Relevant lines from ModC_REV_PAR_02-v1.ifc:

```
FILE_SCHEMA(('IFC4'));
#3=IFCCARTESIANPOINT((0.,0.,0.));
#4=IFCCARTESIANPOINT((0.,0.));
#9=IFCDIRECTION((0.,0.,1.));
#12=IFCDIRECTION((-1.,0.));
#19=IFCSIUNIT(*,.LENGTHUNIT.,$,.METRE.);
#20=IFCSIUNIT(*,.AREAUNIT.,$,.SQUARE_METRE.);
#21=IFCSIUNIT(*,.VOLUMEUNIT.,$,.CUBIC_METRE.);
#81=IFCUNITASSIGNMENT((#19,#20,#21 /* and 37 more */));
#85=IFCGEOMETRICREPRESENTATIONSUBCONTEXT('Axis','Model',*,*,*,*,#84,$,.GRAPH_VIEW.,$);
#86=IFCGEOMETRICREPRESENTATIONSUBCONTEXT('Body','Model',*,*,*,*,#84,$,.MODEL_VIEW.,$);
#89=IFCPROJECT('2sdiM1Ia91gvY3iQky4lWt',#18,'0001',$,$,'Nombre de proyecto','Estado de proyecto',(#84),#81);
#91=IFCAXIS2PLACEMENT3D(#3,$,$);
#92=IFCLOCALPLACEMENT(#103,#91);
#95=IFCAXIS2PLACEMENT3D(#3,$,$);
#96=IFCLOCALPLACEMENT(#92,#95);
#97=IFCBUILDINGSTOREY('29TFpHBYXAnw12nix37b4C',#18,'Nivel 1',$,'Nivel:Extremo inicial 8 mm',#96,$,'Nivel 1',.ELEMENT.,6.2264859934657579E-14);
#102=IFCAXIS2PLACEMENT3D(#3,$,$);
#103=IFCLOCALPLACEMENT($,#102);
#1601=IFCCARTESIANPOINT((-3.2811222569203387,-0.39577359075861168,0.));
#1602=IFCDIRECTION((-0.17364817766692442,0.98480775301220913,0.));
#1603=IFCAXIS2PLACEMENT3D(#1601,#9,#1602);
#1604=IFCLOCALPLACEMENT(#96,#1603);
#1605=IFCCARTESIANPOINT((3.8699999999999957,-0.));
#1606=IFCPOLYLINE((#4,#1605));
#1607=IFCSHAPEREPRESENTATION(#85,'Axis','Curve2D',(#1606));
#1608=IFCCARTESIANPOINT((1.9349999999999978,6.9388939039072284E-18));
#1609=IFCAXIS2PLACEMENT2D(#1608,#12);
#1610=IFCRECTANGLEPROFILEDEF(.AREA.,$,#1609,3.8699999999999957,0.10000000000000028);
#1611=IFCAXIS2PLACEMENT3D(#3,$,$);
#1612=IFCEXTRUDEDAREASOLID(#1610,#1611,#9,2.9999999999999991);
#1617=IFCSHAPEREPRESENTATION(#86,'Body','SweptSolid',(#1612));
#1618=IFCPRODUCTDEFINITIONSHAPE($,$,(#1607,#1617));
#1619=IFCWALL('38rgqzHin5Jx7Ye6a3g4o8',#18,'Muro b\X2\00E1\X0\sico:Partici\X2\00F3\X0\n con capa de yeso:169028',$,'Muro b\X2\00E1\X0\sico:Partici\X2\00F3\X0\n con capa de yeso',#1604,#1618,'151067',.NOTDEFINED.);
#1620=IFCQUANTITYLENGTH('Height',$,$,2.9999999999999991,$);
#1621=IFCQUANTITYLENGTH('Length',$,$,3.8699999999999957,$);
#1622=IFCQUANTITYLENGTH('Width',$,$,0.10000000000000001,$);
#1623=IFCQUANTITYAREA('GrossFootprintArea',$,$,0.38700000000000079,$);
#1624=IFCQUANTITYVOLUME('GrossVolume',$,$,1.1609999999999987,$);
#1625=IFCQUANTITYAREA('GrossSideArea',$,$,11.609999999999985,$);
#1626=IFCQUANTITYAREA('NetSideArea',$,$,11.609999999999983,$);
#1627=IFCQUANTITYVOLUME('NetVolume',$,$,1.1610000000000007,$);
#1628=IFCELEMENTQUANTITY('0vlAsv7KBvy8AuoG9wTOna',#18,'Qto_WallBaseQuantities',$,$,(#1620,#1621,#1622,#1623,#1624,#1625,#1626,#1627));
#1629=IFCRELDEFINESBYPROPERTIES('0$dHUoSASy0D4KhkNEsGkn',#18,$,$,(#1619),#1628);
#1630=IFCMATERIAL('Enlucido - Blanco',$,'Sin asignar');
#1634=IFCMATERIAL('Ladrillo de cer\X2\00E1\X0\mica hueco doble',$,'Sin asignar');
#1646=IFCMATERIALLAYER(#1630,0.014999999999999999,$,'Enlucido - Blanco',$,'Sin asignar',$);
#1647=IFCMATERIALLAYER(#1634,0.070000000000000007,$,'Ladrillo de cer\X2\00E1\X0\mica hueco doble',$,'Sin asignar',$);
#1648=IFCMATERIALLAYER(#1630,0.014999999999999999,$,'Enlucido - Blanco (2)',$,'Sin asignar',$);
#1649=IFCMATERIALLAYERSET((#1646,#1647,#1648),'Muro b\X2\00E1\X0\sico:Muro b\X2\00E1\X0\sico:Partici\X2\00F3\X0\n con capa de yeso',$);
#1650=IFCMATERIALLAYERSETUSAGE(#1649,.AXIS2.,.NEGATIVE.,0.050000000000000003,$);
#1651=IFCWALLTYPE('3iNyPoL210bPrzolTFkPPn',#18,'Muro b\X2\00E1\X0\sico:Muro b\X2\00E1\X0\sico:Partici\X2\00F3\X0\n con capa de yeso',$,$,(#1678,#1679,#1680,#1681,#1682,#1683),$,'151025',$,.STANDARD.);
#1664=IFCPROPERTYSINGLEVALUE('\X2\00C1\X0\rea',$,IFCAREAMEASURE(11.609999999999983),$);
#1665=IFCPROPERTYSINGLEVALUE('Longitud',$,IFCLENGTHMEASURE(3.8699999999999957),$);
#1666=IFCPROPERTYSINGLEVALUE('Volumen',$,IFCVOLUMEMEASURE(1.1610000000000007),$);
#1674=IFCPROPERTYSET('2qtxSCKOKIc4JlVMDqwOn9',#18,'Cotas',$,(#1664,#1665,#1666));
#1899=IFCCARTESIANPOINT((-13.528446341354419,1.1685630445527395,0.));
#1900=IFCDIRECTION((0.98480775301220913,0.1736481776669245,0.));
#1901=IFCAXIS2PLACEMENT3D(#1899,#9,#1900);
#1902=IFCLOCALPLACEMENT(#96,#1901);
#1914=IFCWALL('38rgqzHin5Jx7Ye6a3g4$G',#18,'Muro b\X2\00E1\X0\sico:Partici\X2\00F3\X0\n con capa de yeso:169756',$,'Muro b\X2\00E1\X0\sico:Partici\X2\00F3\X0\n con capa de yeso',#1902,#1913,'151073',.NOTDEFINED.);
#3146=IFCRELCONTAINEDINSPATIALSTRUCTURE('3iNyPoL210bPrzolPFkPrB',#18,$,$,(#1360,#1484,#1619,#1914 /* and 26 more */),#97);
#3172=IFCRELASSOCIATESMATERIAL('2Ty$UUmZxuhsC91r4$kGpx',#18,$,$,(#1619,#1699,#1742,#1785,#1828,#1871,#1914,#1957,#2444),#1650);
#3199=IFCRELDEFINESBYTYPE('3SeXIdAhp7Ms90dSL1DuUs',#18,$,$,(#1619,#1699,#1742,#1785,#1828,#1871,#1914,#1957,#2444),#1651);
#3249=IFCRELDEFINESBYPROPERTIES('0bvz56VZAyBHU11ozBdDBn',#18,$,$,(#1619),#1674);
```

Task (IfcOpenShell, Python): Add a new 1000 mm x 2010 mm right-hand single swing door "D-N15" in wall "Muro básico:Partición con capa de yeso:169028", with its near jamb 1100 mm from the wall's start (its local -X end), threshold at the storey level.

```python
import numpy as np
import ifcopenshell
import ifcopenshell.api.feature
import ifcopenshell.api.geometry
import ifcopenshell.api.pset
import ifcopenshell.api.root
import ifcopenshell.api.spatial
import ifcopenshell.geom
import ifcopenshell.util.element
import ifcopenshell.util.placement
import ifcopenshell.util.representation
import ifcopenshell.util.shape
import ifcopenshell.util.unit

model = ifcopenshell.open("ModC_REV_PAR_02-v1.ifc")
unit_scale = ifcopenshell.util.unit.calculate_unit_scale(model)
area_scale = ifcopenshell.util.unit.calculate_unit_scale(model, "AREAUNIT")
volume_scale = ifcopenshell.util.unit.calculate_unit_scale(model, "VOLUMEUNIT")
settings = ifcopenshell.geom.settings()


def volume(element):
    """Net volume in cubic metres, openings subtracted."""
    shape = ifcopenshell.geom.create_shape(settings, element)
    return ifcopenshell.util.shape.get_volume(shape.geometry)


wall = model.by_guid("38rgqzHin5Jx7Ye6a3g4o8")
storey = ifcopenshell.util.element.get_container(wall, ifc_class="IfcBuildingStorey")
context = ifcopenshell.util.representation.get_context(model, "Model", "Body", "MODEL_VIEW")
before = volume(wall)

width, height, from_end, sill = 1, 2.01, 1.1, 0.0  # metres

# The wall runs along its own X axis, and the end named is its -X end.
wall_shape = ifcopenshell.geom.create_shape(settings, wall)
x, y, z = ifcopenshell.util.shape.get_vertices(wall_shape.geometry).T
start = x.min() + from_end
face, thickness = float(y.min()), float(y.max() - y.min())
wall_matrix = ifcopenshell.util.placement.get_local_placement(wall.ObjectPlacement)
level = ifcopenshell.util.placement.get_local_placement(storey.ObjectPlacement)[2, 3]


def in_wall(x, y):
    """Placement at x, y metres in the wall's axes, at sill height."""
    matrix = wall_matrix.copy()
    matrix[:, 3] = wall_matrix @ np.array([x / unit_scale, y / unit_scale, 0.0, 1.0])
    matrix[2, 3] = level + sill / unit_scale
    return matrix


# Opening: a box that overshoots both wall faces by 50 mm.
opening = ifcopenshell.api.root.create_entity(model, ifc_class="IfcOpeningElement", predefined_type="OPENING")
box = ifcopenshell.api.geometry.add_wall_representation(
    model, context=context, length=width, height=height, thickness=thickness + 0.1
)
ifcopenshell.api.geometry.assign_representation(model, product=opening, representation=box)
ifcopenshell.api.geometry.edit_object_placement(model, product=opening, matrix=in_wall(start, face - 0.05), is_si=False)
ifcopenshell.api.feature.add_feature(model, feature=opening, element=wall)

door = ifcopenshell.api.root.create_entity(model, ifc_class="IfcDoor", name="D-N15", predefined_type="DOOR")
door.OverallWidth, door.OverallHeight = width / unit_scale, height / unit_scale
door.OperationType = "SINGLE_SWING_RIGHT"
body = ifcopenshell.api.geometry.add_door_representation(
    model,
    context=context,
    overall_width=door.OverallWidth,
    overall_height=door.OverallHeight,
    operation_type="SINGLE_SWING_RIGHT",
    lining_properties={"LiningDepth": thickness / unit_scale, "ThresholdDepth": thickness / unit_scale},
)
ifcopenshell.api.geometry.assign_representation(model, product=door, representation=body)
ifcopenshell.api.spatial.assign_container(model, products=[door], relating_structure=storey)
ifcopenshell.api.feature.add_filling(model, opening=opening, element=door)

# The lining spans the wall, so the door starts at the wall face.
ifcopenshell.api.geometry.edit_object_placement(model, product=door, matrix=in_wall(start, face), is_si=False)

after = volume(wall)

# Update the wall's stored quantities.
qto = model.by_id(ifcopenshell.util.element.get_pset(wall, "Qto_WallBaseQuantities", should_inherit=False)["id"])
ifcopenshell.api.pset.edit_qto(model, qto=qto, properties={
    "NetSideArea": after / thickness / area_scale,
    "NetVolume": after / volume_scale,
})
pset = model.by_id(ifcopenshell.util.element.get_pset(wall, "Cotas", should_inherit=False)["id"])
ifcopenshell.api.pset.edit_pset(model, pset=pset, properties={
    "Área": model.create_entity("IfcAreaMeasure", after / thickness / area_scale),
    "Volumen": model.create_entity("IfcVolumeMeasure", after / volume_scale),
})

print(f"wall volume {before:.3f} -> {after:.3f} m3")

model.write("ModC_REV_PAR_02-v1_v2.ifc")
```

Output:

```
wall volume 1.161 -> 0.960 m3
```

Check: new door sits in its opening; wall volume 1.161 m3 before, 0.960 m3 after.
